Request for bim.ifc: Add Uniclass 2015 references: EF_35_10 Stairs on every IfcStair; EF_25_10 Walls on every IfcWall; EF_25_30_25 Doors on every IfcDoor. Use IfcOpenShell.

First a look at what the model holds.

```python
import ifcopenshell

model = ifcopenshell.open("bim.ifc")
print(model.schema)
print("classifications:", [c.Name for c in model.by_type("IfcClassification")])
for ifc_class in ("IfcDoor", "IfcRoof", "IfcStair", "IfcWall", "IfcWindow"):
    print(ifc_class, len(model.by_type(ifc_class)))
```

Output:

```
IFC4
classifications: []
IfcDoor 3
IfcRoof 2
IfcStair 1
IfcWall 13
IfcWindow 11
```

```python
import ifcopenshell
import ifcopenshell.api.classification

model = ifcopenshell.open("bim.ifc")

system = ifcopenshell.api.classification.add_classification(model, classification="Uniclass 2015")

codes = {
    "IfcStair": ("EF_35_10", "Stairs"),
    "IfcWall": ("EF_25_10", "Walls"),
    "IfcDoor": ("EF_25_30_25", "Doors"),
}
for ifc_class, (code, name) in codes.items():
    products = model.by_type(ifc_class)
    ifcopenshell.api.classification.add_reference(
        model, products=products, classification=system, identification=code, name=name
    )
    print(code, len(products))

model.write("bim_edited.ifc")
```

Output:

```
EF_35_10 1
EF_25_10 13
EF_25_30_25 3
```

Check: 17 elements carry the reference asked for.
